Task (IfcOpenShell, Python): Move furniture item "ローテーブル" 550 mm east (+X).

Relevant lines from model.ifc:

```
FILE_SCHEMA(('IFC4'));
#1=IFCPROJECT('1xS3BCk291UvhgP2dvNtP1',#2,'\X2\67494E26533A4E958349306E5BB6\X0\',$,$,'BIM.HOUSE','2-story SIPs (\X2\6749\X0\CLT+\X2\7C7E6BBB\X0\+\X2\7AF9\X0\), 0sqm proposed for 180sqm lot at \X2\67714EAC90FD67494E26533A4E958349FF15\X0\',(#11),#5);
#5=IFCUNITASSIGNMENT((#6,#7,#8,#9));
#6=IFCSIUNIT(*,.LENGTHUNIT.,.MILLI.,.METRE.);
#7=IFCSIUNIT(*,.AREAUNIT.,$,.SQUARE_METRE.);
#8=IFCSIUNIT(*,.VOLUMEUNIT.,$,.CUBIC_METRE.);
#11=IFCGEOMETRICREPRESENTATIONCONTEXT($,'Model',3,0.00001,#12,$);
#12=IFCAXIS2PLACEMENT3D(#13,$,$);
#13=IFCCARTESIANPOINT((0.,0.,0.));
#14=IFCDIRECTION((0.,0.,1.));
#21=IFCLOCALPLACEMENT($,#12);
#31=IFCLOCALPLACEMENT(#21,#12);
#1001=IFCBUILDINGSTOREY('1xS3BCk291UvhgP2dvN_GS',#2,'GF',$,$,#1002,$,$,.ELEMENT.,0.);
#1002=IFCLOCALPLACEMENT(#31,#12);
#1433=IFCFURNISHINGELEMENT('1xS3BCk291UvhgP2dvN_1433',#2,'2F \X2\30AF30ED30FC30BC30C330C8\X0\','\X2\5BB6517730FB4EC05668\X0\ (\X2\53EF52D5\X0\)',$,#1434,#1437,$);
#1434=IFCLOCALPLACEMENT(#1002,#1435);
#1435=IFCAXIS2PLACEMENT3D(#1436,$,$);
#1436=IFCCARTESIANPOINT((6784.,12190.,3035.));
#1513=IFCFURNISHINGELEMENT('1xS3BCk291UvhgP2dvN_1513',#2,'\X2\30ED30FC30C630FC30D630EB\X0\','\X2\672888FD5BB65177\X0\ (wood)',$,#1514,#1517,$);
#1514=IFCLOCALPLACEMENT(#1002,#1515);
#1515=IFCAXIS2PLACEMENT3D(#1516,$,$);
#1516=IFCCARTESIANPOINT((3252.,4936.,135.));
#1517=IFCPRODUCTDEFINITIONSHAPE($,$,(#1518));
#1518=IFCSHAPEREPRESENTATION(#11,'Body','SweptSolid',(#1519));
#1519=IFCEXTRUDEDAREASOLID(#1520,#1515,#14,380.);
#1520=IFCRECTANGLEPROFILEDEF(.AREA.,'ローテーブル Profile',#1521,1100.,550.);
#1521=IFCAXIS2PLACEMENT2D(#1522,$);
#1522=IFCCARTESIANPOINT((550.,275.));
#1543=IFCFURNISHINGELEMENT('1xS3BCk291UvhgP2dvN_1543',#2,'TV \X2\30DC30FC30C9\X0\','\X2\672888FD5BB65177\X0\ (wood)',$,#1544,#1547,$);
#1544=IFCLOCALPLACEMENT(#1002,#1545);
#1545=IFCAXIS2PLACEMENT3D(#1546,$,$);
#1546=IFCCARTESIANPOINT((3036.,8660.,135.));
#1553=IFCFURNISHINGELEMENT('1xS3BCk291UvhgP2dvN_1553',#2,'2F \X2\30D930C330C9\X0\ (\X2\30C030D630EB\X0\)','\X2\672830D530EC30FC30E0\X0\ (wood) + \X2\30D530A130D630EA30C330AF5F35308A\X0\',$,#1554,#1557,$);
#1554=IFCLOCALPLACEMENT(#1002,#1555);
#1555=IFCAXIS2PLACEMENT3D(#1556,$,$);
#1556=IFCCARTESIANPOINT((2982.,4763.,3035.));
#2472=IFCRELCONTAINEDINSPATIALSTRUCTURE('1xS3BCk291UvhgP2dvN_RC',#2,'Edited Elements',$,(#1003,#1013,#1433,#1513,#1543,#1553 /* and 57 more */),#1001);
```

```python
import ifcopenshell
import ifcopenshell.api.geometry
import ifcopenshell.util.placement
import ifcopenshell.util.unit

model = ifcopenshell.open("model.ifc")
unit_scale = ifcopenshell.util.unit.calculate_unit_scale(model)

item = model.by_guid("1xS3BCk291UvhgP2dvN_1513")
matrix = ifcopenshell.util.placement.get_local_placement(item.ObjectPlacement)
matrix[0, 3] += 0.55 / unit_scale
ifcopenshell.api.geometry.edit_object_placement(model, product=item, matrix=matrix, is_si=False)

print(ifcopenshell.util.placement.get_local_placement(item.ObjectPlacement).round(3) + 0.0)

model.write("model-out.ifc")
```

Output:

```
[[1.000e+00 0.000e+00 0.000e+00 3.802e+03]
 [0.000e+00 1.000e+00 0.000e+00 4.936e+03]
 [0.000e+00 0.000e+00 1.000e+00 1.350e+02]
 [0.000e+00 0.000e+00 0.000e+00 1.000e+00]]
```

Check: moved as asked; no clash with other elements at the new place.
